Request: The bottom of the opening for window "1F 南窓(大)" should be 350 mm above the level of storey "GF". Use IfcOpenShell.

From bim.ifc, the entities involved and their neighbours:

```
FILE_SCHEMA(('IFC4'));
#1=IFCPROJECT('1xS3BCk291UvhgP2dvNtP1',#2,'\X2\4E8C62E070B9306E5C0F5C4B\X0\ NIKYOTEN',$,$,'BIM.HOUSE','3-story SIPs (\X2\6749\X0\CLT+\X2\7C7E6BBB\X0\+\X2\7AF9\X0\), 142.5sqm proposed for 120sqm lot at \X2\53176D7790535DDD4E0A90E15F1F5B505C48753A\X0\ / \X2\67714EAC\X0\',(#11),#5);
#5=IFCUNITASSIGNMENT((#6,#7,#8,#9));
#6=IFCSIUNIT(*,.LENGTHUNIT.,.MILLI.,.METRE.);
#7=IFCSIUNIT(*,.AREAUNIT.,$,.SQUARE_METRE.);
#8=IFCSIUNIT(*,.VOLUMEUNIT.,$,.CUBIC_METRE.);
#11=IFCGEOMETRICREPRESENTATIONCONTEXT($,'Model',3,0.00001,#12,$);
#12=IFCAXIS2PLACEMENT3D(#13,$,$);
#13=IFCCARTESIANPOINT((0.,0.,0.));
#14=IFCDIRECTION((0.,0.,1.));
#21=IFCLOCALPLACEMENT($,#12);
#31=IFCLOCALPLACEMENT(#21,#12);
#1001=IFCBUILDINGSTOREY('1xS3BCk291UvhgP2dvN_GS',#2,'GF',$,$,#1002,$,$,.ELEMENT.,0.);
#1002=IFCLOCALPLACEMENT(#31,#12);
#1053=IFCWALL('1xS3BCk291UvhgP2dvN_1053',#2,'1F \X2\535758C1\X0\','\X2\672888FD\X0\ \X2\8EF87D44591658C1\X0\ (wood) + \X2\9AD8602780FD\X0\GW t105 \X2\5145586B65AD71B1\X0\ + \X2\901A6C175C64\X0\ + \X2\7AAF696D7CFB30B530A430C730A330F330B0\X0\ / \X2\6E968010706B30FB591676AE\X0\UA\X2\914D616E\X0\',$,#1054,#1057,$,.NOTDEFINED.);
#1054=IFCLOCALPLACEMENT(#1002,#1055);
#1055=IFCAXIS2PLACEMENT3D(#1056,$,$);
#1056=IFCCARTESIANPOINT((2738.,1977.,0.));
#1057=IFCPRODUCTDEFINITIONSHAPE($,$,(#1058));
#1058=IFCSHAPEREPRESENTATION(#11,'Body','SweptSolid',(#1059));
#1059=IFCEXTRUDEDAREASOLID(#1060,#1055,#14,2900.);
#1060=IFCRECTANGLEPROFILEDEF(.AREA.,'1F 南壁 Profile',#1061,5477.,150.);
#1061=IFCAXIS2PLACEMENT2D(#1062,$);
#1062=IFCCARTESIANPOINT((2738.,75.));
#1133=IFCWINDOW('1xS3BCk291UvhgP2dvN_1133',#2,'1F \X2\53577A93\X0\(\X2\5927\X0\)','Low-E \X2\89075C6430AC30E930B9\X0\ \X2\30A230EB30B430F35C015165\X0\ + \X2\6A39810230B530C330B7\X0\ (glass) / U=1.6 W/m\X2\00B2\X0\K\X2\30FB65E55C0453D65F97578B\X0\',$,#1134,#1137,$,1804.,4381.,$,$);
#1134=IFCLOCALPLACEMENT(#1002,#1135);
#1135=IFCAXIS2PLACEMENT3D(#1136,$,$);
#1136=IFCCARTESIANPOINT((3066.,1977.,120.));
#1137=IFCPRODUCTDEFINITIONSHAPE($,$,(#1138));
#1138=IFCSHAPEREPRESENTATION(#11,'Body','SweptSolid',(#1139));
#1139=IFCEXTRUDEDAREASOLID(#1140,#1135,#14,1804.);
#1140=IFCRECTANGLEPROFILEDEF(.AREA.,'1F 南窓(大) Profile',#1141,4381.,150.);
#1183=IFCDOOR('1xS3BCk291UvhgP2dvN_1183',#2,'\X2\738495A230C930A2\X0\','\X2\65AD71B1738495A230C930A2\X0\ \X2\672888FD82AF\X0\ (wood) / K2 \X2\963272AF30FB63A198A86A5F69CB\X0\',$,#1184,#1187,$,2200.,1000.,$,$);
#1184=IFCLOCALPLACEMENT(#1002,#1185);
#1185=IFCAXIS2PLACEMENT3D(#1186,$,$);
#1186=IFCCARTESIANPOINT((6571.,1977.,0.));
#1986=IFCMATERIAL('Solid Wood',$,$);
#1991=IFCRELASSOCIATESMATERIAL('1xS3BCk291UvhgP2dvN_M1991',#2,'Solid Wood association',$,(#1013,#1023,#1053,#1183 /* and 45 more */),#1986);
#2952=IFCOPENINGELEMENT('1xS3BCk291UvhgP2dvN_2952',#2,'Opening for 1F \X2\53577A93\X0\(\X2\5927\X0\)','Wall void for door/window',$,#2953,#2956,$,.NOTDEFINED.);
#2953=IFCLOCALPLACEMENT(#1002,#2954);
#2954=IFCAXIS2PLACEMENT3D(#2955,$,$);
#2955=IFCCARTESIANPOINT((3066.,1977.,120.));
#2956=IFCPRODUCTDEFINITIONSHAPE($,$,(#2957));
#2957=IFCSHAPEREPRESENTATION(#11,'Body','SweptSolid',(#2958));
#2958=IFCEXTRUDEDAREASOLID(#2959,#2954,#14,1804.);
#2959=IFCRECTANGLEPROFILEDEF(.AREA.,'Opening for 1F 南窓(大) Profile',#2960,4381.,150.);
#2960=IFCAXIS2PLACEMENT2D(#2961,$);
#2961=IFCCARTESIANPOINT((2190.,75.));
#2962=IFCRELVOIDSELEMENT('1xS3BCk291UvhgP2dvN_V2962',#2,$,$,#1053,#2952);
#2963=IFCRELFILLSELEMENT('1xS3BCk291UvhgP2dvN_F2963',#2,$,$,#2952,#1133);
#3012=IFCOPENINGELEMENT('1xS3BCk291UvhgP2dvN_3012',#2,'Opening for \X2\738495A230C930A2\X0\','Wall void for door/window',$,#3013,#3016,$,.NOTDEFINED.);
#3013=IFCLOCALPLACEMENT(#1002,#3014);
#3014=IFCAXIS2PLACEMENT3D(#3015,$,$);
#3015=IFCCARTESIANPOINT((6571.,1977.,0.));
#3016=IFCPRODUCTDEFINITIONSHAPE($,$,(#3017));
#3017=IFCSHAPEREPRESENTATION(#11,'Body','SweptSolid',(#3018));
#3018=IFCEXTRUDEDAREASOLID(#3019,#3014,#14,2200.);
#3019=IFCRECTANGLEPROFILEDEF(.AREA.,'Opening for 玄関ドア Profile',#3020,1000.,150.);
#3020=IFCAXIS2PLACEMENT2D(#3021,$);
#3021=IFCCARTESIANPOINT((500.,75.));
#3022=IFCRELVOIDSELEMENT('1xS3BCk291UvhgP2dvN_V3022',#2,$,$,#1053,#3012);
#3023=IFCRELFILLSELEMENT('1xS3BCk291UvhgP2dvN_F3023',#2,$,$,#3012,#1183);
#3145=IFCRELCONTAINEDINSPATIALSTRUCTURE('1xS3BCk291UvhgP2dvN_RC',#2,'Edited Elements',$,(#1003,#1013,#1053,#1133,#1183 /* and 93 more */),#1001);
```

```python
import numpy as np
import ifcopenshell
import ifcopenshell.api.geometry
import ifcopenshell.geom
import ifcopenshell.util.element
import ifcopenshell.util.placement
import ifcopenshell.util.shape
import ifcopenshell.util.unit

model = ifcopenshell.open("bim.ifc")
unit_scale = ifcopenshell.util.unit.calculate_unit_scale(model)

window = model.by_guid("1xS3BCk291UvhgP2dvN_1133")
opening = window.FillsVoids[0].RelatingOpeningElement
storey = ifcopenshell.util.element.get_container(window, ifc_class="IfcBuildingStorey")
level = ifcopenshell.util.placement.get_local_placement(storey.ObjectPlacement)[2, 3]

# The opening's origin need not be at the sill, so measure its lowest point.
shape = ifcopenshell.geom.create_shape(ifcopenshell.geom.settings(), opening)
bottom = ifcopenshell.util.shape.get_shape_bottom_elevation(shape, shape.geometry) / unit_scale
dz = level + 0.35 / unit_scale - bottom

shift = np.array([0.0, 0.0, dz])
# The window is not placed relative to its opening, so move both.
for product in (opening, window):
    matrix = ifcopenshell.util.placement.get_local_placement(product.ObjectPlacement)
    matrix[:3, 3] += shift
    ifcopenshell.api.geometry.edit_object_placement(model, product=product, matrix=matrix, is_si=False)

print(f"moved by {dz * unit_scale:+.3f} m")

model.write("bim_edited.ifc")
```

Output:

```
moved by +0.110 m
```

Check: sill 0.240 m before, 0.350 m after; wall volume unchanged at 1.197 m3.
